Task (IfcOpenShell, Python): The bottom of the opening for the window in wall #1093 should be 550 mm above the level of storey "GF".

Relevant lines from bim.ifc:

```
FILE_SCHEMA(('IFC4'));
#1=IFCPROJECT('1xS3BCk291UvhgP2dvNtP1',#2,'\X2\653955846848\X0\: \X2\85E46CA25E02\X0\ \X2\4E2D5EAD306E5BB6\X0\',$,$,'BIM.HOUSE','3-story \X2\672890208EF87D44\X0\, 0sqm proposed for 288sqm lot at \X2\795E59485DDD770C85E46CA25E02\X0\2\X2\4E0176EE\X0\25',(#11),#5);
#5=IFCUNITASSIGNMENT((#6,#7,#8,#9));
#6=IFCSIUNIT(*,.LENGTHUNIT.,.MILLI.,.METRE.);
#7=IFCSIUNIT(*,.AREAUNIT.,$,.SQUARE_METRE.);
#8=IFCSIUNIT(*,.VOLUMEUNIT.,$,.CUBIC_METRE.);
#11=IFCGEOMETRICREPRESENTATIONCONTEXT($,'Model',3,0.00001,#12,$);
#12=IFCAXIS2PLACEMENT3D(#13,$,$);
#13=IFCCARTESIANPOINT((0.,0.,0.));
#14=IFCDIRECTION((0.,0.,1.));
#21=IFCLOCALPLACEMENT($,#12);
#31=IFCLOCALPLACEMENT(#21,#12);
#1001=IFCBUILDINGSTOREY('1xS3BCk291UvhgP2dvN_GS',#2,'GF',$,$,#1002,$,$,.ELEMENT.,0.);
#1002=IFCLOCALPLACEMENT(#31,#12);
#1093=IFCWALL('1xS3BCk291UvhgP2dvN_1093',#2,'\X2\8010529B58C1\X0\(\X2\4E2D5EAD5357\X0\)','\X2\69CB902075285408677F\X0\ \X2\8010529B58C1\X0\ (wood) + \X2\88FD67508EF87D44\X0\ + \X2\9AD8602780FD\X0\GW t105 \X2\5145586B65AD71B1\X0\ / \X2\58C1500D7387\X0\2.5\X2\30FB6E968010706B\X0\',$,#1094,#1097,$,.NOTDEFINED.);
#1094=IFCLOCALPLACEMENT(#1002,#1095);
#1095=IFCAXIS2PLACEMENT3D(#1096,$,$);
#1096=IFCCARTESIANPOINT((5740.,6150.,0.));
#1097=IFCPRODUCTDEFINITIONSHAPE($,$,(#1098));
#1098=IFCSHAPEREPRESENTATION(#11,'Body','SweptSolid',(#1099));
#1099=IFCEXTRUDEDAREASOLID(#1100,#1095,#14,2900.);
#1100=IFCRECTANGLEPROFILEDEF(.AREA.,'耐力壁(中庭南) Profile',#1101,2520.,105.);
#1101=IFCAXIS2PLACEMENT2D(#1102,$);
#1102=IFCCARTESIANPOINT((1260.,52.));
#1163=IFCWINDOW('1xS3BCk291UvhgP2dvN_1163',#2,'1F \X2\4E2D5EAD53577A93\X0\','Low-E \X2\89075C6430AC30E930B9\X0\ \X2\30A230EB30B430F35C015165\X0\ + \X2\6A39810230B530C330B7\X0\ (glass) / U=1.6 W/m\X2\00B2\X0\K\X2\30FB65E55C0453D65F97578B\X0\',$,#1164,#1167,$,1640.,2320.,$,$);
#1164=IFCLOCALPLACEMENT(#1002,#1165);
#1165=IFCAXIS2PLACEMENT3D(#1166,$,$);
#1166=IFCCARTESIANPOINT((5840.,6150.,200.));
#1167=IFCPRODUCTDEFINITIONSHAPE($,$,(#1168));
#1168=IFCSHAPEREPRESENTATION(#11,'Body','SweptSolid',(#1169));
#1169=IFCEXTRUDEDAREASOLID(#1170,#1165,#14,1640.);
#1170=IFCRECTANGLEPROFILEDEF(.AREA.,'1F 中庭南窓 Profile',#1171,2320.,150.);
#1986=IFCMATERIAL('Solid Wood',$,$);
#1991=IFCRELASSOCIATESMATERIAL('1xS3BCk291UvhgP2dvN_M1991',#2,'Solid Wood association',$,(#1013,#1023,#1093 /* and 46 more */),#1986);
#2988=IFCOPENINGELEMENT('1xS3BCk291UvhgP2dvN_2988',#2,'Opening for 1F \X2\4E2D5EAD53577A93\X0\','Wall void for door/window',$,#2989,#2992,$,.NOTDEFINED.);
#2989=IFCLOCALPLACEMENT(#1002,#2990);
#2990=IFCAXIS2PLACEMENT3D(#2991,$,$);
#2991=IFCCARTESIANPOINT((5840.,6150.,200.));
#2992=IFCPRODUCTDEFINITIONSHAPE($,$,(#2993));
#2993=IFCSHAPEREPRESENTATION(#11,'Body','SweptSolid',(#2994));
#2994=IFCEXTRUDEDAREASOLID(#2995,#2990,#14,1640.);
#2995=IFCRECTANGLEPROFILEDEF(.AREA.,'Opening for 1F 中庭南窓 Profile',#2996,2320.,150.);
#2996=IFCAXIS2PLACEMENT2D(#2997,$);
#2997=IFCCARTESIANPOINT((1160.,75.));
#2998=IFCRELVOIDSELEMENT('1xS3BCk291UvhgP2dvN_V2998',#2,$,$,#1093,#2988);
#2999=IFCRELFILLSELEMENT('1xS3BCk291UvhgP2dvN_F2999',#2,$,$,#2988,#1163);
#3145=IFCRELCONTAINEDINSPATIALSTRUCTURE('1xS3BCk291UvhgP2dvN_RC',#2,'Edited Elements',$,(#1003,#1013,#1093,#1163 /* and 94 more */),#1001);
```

```python
import numpy as np
import ifcopenshell
import ifcopenshell.api.geometry
import ifcopenshell.geom
import ifcopenshell.util.element
import ifcopenshell.util.placement
import ifcopenshell.util.shape
import ifcopenshell.util.unit

model = ifcopenshell.open("bim.ifc")
unit_scale = ifcopenshell.util.unit.calculate_unit_scale(model)

window = model.by_guid("1xS3BCk291UvhgP2dvN_1163")
opening = window.FillsVoids[0].RelatingOpeningElement
storey = ifcopenshell.util.element.get_container(window, ifc_class="IfcBuildingStorey")
level = ifcopenshell.util.placement.get_local_placement(storey.ObjectPlacement)[2, 3]

# The opening's origin need not be at the sill, so measure its lowest point.
shape = ifcopenshell.geom.create_shape(ifcopenshell.geom.settings(), opening)
bottom = ifcopenshell.util.shape.get_shape_bottom_elevation(shape, shape.geometry) / unit_scale
dz = level + 550.0 - bottom

shift = np.array([0.0, 0.0, dz])
# The window is not placed relative to its opening, so move both.
for product in (opening, window):
    matrix = ifcopenshell.util.placement.get_local_placement(product.ObjectPlacement)
    matrix[:3, 3] += shift
    ifcopenshell.api.geometry.edit_object_placement(model, product=product, matrix=matrix, is_si=False)

print(f"moved by {dz * unit_scale:+.3f} m")

model.write("bim_rev.ifc")
```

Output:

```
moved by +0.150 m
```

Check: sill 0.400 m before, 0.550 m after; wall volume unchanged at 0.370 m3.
